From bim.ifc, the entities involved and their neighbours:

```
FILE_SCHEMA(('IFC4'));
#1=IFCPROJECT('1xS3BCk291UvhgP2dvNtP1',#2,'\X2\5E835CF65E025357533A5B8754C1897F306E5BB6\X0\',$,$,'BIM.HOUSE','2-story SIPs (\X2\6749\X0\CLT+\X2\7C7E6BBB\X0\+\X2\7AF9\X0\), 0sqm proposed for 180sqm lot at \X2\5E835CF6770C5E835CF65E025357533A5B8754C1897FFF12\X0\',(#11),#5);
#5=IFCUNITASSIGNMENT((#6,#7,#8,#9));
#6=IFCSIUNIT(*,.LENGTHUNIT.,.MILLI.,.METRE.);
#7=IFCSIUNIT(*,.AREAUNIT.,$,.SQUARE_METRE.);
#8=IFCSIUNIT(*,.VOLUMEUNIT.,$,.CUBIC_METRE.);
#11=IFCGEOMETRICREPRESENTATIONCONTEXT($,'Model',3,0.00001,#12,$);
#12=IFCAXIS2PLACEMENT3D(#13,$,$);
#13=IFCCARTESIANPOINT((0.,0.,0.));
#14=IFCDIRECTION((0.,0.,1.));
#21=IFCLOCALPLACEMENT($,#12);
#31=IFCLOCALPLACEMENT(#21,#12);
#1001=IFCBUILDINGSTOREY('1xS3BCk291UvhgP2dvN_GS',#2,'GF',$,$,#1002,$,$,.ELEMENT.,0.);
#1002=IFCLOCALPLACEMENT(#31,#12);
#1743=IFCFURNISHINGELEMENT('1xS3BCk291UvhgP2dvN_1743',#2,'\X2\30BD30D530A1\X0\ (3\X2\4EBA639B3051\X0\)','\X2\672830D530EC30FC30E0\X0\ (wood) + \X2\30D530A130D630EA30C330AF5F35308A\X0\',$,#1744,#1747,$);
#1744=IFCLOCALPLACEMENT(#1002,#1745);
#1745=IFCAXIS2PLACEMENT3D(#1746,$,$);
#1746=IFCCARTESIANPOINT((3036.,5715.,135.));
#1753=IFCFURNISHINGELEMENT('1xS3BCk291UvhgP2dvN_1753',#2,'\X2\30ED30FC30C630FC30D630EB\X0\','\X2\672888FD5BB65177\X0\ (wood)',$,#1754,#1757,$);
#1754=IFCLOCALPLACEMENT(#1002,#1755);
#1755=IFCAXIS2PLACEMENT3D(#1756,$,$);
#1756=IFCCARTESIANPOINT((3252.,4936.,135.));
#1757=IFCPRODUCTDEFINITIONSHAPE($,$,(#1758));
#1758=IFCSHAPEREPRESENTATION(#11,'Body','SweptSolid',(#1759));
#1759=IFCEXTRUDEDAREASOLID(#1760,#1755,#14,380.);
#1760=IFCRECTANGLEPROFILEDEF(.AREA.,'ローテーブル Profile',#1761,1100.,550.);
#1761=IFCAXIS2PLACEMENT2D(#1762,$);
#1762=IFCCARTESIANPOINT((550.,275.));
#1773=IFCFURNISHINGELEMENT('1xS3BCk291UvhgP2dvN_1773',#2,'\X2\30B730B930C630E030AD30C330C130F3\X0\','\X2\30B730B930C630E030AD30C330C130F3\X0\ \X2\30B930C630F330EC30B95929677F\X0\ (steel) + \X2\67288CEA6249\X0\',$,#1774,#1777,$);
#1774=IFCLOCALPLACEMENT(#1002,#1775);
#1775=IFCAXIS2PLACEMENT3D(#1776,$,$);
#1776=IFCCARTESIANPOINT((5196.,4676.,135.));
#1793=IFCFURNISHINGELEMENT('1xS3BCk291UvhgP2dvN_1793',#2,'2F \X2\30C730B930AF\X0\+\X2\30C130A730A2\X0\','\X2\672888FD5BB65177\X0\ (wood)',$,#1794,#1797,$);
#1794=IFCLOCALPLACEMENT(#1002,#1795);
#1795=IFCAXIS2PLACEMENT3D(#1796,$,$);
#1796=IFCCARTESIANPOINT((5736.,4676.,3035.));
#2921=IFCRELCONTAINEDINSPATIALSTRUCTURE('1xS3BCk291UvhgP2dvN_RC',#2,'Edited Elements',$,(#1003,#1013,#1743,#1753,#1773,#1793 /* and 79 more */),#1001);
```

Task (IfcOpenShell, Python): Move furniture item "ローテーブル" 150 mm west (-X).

```python
import ifcopenshell
import ifcopenshell.api.geometry
import ifcopenshell.util.placement

model = ifcopenshell.open("bim.ifc")

item = model.by_guid("1xS3BCk291UvhgP2dvN_1753")
matrix = ifcopenshell.util.placement.get_local_placement(item.ObjectPlacement)
matrix[0, 3] -= 150.0
ifcopenshell.api.geometry.edit_object_placement(model, product=item, matrix=matrix, is_si=False)

print(ifcopenshell.util.placement.get_local_placement(item.ObjectPlacement).round(3) + 0.0)

model.write("bim_v2.ifc")
```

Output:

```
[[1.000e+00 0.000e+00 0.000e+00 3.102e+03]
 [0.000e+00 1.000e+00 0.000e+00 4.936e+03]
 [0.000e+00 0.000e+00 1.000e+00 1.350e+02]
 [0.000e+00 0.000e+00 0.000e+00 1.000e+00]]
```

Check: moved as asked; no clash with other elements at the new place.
